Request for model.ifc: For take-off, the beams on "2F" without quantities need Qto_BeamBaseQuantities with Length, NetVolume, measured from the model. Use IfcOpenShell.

First a look at what the model holds.

```python
import ifcopenshell
import ifcopenshell.util.element
import ifcopenshell.util.unit

model = ifcopenshell.open("model.ifc")
print(model.schema)
for unit_type in ("LENGTHUNIT", "AREAUNIT", "VOLUMEUNIT"):
    print(unit_type, ifcopenshell.util.unit.calculate_unit_scale(model, unit_type))
storey = next(s for s in model.by_type("IfcBuildingStorey") if s.Name == "2F")
beams = [e for e in ifcopenshell.util.element.get_decomposition(storey) if e.is_a("IfcBeam")]
for e in sorted(beams, key=lambda e: e.id()):
    print(e.id(), e.is_a(), e.Name, list(ifcopenshell.util.element.get_psets(e, qtos_only=True)), sep=" | ")
```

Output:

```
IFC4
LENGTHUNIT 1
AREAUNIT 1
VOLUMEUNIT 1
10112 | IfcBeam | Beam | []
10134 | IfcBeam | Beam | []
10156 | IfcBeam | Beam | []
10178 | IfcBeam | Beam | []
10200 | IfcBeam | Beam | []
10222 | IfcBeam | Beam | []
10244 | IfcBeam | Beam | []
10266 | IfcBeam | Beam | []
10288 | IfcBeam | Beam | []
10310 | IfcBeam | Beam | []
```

```python
import ifcopenshell
import ifcopenshell.api.pset
import ifcopenshell.geom
import ifcopenshell.util.element
import ifcopenshell.util.shape
import ifcopenshell.util.unit

model = ifcopenshell.open("model.ifc")
unit_scale = ifcopenshell.util.unit.calculate_unit_scale(model)
volume_scale = ifcopenshell.util.unit.calculate_unit_scale(model, "VOLUMEUNIT")
settings = ifcopenshell.geom.settings()

storey = next(s for s in model.by_type("IfcBuildingStorey") if s.Name == "2F")
beams = [e for e in ifcopenshell.util.element.get_decomposition(storey) if e.is_a("IfcBeam")]

for e in sorted(beams, key=lambda e: e.id()):
    if ifcopenshell.util.element.get_psets(e, qtos_only=True, should_inherit=False):
        continue
    # Geometry comes back in metres, in the element's own axes.
    shape = ifcopenshell.geom.create_shape(settings, e)
    values = {
        "Length": ifcopenshell.util.shape.get_max_xyz(shape.geometry) / unit_scale,
        "NetVolume": ifcopenshell.util.shape.get_volume(shape.geometry) / volume_scale,
    }
    qto = ifcopenshell.api.pset.add_qto(model, product=e, name="Qto_BeamBaseQuantities")
    ifcopenshell.api.pset.edit_qto(model, qto=qto, properties=values)
    print(e.id(), {k: round(v, 3) for k, v in values.items()})

model.write("model_v2.ifc")
```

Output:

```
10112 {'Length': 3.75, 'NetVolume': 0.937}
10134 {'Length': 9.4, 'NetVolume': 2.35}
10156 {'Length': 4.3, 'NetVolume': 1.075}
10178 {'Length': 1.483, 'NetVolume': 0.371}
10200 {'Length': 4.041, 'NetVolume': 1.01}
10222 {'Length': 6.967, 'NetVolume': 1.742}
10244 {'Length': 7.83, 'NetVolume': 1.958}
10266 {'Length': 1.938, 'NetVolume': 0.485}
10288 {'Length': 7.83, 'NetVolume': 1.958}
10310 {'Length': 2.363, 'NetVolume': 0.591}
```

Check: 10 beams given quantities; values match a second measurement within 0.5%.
